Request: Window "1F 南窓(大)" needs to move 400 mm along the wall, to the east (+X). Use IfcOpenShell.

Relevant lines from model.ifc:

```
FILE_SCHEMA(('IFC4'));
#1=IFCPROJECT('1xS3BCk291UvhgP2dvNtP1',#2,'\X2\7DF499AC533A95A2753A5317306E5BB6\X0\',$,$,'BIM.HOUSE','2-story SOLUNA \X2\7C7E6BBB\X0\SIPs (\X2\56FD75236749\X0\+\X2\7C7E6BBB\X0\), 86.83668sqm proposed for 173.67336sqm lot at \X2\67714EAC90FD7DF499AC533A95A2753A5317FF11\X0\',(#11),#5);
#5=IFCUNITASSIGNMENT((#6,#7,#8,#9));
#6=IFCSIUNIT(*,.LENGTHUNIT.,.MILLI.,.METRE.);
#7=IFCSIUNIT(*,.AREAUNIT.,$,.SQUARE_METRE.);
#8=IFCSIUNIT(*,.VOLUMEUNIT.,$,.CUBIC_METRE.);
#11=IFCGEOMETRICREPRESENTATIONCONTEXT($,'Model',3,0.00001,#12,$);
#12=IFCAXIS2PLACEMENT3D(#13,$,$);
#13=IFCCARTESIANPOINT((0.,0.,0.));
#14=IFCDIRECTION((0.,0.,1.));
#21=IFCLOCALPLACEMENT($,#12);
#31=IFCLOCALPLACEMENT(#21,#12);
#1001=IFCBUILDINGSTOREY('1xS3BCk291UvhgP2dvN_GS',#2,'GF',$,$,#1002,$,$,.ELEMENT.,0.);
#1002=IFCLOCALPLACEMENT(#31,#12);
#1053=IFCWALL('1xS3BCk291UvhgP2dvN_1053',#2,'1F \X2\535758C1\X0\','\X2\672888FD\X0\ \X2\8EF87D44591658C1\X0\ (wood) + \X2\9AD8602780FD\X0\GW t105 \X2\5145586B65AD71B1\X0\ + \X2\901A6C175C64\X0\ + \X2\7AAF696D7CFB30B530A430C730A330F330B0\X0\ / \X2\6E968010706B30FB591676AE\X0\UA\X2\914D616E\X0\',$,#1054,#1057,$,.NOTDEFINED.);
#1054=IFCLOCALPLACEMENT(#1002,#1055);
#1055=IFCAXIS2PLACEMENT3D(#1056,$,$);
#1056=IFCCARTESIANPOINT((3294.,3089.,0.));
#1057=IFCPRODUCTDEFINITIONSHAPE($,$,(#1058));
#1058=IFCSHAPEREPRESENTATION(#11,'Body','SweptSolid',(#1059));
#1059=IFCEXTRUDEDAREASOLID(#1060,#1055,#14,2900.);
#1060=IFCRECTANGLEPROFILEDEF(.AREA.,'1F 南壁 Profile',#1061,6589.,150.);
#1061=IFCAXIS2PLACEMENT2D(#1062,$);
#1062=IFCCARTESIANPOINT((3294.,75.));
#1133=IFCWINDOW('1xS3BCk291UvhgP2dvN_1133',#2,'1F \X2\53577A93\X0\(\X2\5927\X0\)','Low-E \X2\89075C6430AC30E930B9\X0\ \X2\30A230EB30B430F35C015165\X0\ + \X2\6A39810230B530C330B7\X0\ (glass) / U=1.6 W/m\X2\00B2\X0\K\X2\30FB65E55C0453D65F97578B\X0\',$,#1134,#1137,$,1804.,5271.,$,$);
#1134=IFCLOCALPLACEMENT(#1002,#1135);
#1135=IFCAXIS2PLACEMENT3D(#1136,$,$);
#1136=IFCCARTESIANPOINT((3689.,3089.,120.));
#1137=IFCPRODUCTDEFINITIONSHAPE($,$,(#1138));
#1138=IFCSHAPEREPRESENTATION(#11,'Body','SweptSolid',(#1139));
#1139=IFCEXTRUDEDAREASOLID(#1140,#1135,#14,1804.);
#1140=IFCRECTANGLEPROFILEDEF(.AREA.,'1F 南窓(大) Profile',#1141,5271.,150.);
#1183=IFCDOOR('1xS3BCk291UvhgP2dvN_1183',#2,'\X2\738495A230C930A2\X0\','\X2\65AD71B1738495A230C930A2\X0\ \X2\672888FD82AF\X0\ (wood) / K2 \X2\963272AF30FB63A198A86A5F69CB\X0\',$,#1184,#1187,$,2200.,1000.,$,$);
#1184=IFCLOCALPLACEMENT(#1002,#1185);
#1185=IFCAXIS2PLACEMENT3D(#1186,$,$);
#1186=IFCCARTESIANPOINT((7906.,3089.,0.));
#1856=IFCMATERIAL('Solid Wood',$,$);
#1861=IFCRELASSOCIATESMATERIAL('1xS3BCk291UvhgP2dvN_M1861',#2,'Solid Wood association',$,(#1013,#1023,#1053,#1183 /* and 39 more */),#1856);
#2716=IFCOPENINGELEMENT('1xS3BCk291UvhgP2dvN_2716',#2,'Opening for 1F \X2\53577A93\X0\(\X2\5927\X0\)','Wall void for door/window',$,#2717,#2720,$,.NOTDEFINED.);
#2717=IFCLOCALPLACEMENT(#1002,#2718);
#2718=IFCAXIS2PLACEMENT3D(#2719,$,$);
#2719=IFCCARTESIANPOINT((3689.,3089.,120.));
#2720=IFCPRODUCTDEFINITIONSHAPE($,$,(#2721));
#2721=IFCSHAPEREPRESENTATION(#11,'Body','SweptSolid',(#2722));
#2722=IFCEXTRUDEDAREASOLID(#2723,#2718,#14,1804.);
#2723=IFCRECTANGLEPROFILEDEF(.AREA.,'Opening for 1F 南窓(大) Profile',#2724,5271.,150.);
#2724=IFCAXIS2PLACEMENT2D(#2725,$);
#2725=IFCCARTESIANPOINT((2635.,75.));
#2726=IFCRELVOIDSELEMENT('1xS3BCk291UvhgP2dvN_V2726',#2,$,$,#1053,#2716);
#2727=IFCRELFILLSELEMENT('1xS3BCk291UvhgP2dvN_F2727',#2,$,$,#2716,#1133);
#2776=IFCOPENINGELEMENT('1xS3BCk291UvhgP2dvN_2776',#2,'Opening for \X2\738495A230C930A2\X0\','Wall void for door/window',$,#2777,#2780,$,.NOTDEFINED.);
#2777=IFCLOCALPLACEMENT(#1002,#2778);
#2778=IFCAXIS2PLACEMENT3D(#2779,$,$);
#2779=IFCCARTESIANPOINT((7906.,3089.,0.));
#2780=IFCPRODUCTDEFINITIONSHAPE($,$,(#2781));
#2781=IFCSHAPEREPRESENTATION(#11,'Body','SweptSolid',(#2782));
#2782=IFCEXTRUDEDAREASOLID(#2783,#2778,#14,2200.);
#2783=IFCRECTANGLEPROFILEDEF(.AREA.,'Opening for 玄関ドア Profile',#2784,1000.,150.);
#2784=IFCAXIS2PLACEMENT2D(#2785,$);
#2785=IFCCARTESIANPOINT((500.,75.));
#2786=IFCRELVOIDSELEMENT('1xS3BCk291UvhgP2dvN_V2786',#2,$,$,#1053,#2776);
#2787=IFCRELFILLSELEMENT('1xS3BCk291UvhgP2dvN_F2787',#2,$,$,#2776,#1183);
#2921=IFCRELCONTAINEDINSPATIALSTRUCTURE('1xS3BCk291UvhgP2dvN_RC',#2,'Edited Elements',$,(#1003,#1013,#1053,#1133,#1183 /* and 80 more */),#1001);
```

```python
import ifcopenshell
import ifcopenshell.api.geometry
import ifcopenshell.util.placement
import ifcopenshell.util.unit

model = ifcopenshell.open("model.ifc")
unit_scale = ifcopenshell.util.unit.calculate_unit_scale(model)

window = model.by_guid("1xS3BCk291UvhgP2dvN_1133")
opening = window.FillsVoids[0].RelatingOpeningElement
wall = opening.VoidsElements[0].RelatingBuildingElement

wall_matrix = ifcopenshell.util.placement.get_local_placement(wall.ObjectPlacement)
shift = wall_matrix[:3, 0] * 0.4 / unit_scale
before = ifcopenshell.util.placement.get_local_placement(window.ObjectPlacement)[:3, 3].copy()

# The window is not placed relative to its opening, so move both.
for product in (opening, window):
    matrix = ifcopenshell.util.placement.get_local_placement(product.ObjectPlacement)
    matrix[:3, 3] += shift
    ifcopenshell.api.geometry.edit_object_placement(model, product=product, matrix=matrix, is_si=False)

after = ifcopenshell.util.placement.get_local_placement(window.ObjectPlacement)[:3, 3]
print("window moved by", (after - before).round(3) + 0.0)

model.write("model_updated.ifc")
```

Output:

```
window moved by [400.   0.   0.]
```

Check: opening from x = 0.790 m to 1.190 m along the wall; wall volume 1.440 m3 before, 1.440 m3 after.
